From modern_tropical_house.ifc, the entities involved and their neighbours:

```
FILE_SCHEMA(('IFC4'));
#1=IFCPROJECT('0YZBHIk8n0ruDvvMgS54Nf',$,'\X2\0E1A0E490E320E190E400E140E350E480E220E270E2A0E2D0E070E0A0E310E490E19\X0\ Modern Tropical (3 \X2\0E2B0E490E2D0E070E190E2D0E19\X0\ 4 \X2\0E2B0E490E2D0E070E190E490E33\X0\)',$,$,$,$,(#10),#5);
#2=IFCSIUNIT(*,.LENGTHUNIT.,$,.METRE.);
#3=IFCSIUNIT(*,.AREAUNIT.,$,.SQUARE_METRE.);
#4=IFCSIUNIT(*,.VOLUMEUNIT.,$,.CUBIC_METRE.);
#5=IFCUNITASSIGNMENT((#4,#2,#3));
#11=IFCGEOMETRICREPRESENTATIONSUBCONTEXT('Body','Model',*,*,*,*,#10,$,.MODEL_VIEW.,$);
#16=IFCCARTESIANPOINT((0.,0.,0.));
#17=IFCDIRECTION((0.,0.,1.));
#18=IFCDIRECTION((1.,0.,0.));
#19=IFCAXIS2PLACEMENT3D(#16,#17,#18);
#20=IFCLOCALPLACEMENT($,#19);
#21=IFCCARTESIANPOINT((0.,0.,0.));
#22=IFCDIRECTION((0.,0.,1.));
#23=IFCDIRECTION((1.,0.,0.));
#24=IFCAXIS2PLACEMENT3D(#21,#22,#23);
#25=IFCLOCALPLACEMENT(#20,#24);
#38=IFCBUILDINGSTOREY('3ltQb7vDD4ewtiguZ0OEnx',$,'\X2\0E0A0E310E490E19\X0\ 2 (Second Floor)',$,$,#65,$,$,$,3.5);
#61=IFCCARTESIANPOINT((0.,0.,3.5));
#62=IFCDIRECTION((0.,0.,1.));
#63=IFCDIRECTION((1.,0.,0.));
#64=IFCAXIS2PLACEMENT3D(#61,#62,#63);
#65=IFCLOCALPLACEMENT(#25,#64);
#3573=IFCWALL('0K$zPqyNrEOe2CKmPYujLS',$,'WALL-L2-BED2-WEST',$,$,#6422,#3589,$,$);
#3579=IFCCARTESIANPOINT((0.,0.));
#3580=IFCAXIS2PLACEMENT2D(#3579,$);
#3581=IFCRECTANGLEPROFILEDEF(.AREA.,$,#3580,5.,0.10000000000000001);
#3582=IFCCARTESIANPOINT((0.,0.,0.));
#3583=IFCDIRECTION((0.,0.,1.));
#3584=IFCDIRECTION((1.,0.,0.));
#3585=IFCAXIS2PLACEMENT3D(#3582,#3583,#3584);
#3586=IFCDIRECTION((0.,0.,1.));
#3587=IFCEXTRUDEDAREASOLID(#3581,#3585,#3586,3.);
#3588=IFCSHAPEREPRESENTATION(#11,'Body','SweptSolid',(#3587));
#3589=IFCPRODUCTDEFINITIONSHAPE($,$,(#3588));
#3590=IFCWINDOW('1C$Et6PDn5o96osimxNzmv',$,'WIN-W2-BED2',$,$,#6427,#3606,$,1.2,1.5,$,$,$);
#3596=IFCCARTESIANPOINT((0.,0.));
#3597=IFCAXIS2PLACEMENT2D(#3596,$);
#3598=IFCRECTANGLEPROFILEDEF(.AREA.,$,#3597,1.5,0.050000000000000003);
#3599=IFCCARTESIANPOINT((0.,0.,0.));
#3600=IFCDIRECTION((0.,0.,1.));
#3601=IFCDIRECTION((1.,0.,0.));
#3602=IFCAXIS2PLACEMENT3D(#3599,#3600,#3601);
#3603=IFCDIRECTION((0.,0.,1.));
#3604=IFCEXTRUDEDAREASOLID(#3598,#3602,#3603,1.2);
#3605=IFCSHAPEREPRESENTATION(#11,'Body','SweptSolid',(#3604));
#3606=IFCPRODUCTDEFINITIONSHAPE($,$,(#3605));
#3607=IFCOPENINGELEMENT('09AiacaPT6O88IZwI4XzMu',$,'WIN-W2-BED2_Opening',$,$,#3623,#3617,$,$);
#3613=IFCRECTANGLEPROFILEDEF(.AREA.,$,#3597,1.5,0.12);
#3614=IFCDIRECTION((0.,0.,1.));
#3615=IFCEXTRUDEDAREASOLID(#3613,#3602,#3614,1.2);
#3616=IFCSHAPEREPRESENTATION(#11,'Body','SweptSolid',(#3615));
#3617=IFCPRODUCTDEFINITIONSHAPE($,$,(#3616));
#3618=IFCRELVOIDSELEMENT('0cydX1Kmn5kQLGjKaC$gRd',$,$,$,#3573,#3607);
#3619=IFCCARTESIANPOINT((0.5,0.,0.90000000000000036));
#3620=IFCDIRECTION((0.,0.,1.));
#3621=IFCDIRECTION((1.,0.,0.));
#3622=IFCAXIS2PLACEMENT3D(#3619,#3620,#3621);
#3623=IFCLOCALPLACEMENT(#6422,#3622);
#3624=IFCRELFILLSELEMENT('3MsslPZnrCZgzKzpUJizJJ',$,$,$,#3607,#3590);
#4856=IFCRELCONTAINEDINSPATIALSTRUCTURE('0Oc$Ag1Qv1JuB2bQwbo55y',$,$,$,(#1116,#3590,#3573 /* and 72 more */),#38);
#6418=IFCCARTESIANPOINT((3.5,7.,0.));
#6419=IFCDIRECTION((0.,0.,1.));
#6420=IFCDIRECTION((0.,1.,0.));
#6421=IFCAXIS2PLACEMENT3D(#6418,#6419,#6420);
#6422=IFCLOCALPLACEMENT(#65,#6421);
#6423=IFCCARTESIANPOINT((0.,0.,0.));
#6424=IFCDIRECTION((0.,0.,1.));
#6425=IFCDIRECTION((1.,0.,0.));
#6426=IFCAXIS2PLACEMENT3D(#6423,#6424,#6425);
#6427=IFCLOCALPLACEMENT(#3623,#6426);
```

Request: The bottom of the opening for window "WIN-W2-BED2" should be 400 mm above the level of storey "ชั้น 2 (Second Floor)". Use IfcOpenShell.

```python
import numpy as np
import ifcopenshell
import ifcopenshell.api.geometry
import ifcopenshell.geom
import ifcopenshell.util.element
import ifcopenshell.util.placement
import ifcopenshell.util.shape
import ifcopenshell.util.unit

model = ifcopenshell.open("modern_tropical_house.ifc")
unit_scale = ifcopenshell.util.unit.calculate_unit_scale(model)

window = model.by_id(3590)
opening = window.FillsVoids[0].RelatingOpeningElement
storey = ifcopenshell.util.element.get_container(window, ifc_class="IfcBuildingStorey")
level = ifcopenshell.util.placement.get_local_placement(storey.ObjectPlacement)[2, 3]

# The opening's origin need not be at the sill, so measure its lowest point.
shape = ifcopenshell.geom.create_shape(ifcopenshell.geom.settings(), opening)
bottom = ifcopenshell.util.shape.get_shape_bottom_elevation(shape, shape.geometry) / unit_scale
dz = level + 0.4 / unit_scale - bottom

shift = np.array([0.0, 0.0, dz])
# The window is placed relative to its opening, so it follows when the opening moves.
matrix = ifcopenshell.util.placement.get_local_placement(opening.ObjectPlacement)
matrix[:3, 3] += shift
ifcopenshell.api.geometry.edit_object_placement(
    model, product=opening, matrix=matrix, is_si=False, should_transform_children=True
)

print(f"moved by {dz * unit_scale:+.3f} m")

model.write("modern_tropical_house_updated.ifc")
```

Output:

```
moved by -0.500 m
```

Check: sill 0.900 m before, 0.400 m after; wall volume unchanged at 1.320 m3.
